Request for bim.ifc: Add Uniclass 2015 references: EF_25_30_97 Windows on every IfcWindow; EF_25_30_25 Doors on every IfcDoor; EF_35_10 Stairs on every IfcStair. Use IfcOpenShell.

First a look at what the model holds.

```python
import ifcopenshell

model = ifcopenshell.open("bim.ifc")
print(model.schema)
print("classifications:", [c.Name for c in model.by_type("IfcClassification")])
for ifc_class in ("IfcDoor", "IfcRoof", "IfcStair", "IfcWall", "IfcWindow"):
    print(ifc_class, len(model.by_type(ifc_class)))
```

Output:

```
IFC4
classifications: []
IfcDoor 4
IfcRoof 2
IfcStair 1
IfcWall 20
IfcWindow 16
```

```python
import ifcopenshell
import ifcopenshell.api.classification

model = ifcopenshell.open("bim.ifc")

system = ifcopenshell.api.classification.add_classification(model, classification="Uniclass 2015")

codes = {
    "IfcWindow": ("EF_25_30_97", "Windows"),
    "IfcDoor": ("EF_25_30_25", "Doors"),
    "IfcStair": ("EF_35_10", "Stairs"),
}
for ifc_class, (code, name) in codes.items():
    products = model.by_type(ifc_class)
    ifcopenshell.api.classification.add_reference(
        model, products=products, classification=system, identification=code, name=name
    )
    print(code, len(products))

model.write("bim_v2.ifc")
```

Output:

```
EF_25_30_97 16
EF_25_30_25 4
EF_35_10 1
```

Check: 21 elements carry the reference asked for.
